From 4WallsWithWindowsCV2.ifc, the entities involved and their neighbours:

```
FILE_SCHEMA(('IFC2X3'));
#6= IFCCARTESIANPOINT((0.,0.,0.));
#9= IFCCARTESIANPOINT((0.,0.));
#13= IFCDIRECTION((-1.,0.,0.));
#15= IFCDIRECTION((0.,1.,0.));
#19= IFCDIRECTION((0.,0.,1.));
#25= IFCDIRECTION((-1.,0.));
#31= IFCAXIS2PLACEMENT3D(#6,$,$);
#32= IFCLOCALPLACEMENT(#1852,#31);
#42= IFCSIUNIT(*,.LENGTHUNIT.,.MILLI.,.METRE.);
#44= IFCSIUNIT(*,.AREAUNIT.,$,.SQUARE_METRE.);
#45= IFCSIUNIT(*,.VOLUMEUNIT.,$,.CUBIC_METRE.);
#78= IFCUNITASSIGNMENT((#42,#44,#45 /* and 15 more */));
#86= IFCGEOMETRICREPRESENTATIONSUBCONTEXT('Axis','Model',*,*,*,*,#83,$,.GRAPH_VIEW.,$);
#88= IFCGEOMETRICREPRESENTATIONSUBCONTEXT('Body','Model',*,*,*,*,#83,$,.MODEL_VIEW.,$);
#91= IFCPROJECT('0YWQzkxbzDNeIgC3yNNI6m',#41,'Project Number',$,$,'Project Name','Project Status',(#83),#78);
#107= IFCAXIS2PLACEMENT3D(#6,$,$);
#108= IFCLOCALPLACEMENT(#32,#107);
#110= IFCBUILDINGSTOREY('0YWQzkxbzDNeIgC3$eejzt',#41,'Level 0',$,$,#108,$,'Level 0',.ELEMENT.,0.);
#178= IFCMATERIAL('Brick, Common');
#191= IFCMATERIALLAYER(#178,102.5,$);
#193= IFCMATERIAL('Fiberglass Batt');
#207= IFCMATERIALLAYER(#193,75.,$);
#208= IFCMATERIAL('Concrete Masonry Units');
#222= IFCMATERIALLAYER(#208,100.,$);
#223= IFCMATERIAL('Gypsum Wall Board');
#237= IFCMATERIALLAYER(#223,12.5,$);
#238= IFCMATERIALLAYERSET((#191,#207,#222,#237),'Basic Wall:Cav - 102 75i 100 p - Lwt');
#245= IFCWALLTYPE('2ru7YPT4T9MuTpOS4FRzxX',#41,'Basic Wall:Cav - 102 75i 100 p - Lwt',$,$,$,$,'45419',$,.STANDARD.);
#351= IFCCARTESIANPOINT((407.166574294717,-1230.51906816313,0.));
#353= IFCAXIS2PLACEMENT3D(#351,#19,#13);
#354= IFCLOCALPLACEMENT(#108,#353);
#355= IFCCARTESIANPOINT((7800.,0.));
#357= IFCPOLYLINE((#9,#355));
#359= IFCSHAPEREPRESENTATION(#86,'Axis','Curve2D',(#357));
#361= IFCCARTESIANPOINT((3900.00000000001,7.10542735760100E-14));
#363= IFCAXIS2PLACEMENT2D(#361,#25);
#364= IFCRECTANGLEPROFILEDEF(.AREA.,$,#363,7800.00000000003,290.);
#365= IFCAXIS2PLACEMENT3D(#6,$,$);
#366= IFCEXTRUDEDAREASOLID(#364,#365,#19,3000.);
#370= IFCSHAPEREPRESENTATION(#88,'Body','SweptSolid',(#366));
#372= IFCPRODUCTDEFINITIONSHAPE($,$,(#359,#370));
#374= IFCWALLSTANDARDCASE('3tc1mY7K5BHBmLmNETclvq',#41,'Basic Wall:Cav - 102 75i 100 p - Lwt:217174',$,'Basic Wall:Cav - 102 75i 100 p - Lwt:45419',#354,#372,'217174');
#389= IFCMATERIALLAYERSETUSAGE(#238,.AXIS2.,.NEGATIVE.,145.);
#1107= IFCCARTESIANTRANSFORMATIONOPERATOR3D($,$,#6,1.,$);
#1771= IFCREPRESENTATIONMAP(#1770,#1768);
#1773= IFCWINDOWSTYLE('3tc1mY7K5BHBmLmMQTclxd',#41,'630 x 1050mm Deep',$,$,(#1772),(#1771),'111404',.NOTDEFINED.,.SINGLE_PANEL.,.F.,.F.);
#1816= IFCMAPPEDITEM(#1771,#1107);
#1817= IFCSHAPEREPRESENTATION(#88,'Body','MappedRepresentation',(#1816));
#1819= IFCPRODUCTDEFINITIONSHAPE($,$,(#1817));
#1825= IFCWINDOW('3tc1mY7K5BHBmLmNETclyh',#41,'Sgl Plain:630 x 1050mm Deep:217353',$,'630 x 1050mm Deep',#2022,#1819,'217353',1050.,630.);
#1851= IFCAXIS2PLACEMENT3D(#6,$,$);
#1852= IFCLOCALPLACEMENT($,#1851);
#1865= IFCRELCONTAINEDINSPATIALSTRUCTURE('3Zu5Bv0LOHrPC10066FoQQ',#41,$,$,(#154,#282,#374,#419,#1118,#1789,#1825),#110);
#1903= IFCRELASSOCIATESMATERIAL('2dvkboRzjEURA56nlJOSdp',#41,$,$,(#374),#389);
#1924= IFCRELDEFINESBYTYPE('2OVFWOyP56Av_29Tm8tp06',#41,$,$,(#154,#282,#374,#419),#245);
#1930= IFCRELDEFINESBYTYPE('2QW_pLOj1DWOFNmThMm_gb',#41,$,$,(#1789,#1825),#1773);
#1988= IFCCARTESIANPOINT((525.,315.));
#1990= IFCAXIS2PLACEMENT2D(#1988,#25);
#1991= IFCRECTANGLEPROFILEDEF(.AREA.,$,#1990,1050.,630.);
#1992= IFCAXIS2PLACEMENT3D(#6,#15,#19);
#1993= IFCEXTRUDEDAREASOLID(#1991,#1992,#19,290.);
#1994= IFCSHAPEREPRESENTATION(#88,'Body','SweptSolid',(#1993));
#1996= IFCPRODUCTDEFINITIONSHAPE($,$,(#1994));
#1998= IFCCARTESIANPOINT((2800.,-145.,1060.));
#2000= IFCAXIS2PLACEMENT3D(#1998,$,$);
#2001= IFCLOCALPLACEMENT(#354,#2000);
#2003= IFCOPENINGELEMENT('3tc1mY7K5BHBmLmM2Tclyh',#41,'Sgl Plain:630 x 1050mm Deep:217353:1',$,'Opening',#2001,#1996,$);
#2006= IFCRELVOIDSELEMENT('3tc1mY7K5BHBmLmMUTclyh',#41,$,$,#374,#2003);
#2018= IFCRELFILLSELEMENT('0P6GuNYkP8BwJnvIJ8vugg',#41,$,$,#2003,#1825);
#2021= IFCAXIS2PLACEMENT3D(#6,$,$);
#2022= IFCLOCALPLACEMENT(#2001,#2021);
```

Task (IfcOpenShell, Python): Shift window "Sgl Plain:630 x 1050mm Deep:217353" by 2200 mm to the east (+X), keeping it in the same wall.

```python
import ifcopenshell
import ifcopenshell.api.geometry
import ifcopenshell.util.placement

model = ifcopenshell.open("4WallsWithWindowsCV2.ifc")

window = model.by_id(1825)
opening = window.FillsVoids[0].RelatingOpeningElement
wall = opening.VoidsElements[0].RelatingBuildingElement

wall_matrix = ifcopenshell.util.placement.get_local_placement(wall.ObjectPlacement)
shift = wall_matrix[:3, 0] * -2200.0
before = ifcopenshell.util.placement.get_local_placement(window.ObjectPlacement)[:3, 3].copy()

# The window is placed relative to its opening, so it follows when the opening moves.
matrix = ifcopenshell.util.placement.get_local_placement(opening.ObjectPlacement)
matrix[:3, 3] += shift
ifcopenshell.api.geometry.edit_object_placement(
    model, product=opening, matrix=matrix, is_si=False, should_transform_children=True
)

after = ifcopenshell.util.placement.get_local_placement(window.ObjectPlacement)[:3, 3]
print("window moved by", (after - before).round(3) + 0.0)

model.write("4WallsWithWindowsCV2_updated.ifc")
```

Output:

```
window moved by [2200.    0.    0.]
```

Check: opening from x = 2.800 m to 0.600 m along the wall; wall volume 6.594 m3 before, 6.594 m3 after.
